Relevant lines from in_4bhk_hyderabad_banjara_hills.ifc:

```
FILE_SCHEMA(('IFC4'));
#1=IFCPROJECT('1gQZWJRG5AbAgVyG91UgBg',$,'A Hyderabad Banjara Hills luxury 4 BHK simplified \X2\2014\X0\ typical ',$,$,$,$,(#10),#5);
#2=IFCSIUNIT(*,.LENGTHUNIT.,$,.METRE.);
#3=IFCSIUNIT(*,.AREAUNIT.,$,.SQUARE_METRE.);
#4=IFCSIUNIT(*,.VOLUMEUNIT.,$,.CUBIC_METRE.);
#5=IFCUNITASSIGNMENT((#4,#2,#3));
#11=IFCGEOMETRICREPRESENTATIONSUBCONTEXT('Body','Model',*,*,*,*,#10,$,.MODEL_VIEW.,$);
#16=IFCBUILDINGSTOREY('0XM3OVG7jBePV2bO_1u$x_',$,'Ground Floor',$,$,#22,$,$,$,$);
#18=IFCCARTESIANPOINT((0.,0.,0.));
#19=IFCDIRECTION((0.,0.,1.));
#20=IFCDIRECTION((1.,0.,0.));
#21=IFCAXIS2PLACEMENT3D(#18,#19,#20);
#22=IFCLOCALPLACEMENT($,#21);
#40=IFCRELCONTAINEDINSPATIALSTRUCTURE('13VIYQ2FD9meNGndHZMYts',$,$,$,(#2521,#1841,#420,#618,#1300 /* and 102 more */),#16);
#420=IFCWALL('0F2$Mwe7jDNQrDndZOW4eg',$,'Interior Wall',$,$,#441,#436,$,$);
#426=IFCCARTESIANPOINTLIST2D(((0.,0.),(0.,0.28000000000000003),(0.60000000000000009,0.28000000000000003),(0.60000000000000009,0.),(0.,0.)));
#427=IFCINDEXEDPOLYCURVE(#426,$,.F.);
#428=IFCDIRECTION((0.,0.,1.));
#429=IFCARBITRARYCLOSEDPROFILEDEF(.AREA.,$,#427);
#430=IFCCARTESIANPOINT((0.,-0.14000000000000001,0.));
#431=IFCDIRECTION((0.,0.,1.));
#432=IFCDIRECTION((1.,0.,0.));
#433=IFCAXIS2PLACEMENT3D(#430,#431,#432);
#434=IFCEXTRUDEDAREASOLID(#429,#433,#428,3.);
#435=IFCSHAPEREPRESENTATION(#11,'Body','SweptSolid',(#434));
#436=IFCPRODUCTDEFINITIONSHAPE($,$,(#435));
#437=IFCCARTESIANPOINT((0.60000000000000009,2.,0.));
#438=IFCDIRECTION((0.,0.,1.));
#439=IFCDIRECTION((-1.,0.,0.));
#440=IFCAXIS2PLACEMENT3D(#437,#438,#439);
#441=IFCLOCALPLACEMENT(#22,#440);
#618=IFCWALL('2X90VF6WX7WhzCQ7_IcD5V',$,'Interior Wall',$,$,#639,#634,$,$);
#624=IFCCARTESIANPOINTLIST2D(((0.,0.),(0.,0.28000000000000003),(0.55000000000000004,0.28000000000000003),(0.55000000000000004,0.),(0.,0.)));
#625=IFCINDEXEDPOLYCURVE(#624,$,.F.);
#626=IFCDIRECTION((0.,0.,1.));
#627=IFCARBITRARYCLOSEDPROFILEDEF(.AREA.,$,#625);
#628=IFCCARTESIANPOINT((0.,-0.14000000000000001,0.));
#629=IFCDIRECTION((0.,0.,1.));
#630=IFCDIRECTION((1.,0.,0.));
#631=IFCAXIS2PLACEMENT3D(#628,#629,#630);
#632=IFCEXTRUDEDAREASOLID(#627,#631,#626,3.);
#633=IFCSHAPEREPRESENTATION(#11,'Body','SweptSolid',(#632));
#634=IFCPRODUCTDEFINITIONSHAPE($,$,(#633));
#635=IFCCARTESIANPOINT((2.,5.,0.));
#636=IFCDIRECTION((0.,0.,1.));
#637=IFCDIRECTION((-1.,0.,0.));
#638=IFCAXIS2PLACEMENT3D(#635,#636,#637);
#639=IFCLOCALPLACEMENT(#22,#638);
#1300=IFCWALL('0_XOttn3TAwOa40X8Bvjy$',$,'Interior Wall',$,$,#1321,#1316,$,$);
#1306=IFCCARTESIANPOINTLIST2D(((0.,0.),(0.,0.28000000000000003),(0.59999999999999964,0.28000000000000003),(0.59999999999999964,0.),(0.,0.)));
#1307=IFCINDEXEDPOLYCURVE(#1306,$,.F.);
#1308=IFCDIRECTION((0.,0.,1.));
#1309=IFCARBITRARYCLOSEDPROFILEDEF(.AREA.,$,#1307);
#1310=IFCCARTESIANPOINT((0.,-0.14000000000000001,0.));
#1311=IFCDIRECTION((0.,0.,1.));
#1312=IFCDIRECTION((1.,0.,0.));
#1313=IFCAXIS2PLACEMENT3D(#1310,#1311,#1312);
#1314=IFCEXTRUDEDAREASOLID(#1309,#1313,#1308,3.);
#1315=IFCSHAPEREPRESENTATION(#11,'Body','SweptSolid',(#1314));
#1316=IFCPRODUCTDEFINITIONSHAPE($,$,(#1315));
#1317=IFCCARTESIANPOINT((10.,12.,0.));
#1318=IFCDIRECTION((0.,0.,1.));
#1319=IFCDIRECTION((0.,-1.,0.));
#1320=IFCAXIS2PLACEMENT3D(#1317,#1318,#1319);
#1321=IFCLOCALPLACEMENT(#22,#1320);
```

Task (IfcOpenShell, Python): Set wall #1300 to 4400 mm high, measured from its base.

```python
import ifcopenshell
import ifcopenshell.geom
import ifcopenshell.util.representation
import ifcopenshell.util.shape
import ifcopenshell.util.unit

model = ifcopenshell.open("in_4bhk_hyderabad_banjara_hills.ifc")
unit_scale = ifcopenshell.util.unit.calculate_unit_scale(model)
settings = ifcopenshell.geom.settings()


def volume(element):
    """Net volume in cubic metres, openings subtracted."""
    shape = ifcopenshell.geom.create_shape(settings, element)
    return ifcopenshell.util.shape.get_volume(shape.geometry)


wall = model.by_guid("0_XOttn3TAwOa40X8Bvjy$")
before = volume(wall)

body = ifcopenshell.util.representation.get_representation(wall, "Model", "Body")
solid = body.Items[0]
old_height = solid.Depth
solid.Depth = 4.4 / unit_scale
after = volume(wall)

print(f"height {old_height:g} -> {solid.Depth:g}, volume {before:.3f} -> {after:.3f} m3")

model.write("in_4bhk_hyderabad_banjara_hills_v2.ifc")
```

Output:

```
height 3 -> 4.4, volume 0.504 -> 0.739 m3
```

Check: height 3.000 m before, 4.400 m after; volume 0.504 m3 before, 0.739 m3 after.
